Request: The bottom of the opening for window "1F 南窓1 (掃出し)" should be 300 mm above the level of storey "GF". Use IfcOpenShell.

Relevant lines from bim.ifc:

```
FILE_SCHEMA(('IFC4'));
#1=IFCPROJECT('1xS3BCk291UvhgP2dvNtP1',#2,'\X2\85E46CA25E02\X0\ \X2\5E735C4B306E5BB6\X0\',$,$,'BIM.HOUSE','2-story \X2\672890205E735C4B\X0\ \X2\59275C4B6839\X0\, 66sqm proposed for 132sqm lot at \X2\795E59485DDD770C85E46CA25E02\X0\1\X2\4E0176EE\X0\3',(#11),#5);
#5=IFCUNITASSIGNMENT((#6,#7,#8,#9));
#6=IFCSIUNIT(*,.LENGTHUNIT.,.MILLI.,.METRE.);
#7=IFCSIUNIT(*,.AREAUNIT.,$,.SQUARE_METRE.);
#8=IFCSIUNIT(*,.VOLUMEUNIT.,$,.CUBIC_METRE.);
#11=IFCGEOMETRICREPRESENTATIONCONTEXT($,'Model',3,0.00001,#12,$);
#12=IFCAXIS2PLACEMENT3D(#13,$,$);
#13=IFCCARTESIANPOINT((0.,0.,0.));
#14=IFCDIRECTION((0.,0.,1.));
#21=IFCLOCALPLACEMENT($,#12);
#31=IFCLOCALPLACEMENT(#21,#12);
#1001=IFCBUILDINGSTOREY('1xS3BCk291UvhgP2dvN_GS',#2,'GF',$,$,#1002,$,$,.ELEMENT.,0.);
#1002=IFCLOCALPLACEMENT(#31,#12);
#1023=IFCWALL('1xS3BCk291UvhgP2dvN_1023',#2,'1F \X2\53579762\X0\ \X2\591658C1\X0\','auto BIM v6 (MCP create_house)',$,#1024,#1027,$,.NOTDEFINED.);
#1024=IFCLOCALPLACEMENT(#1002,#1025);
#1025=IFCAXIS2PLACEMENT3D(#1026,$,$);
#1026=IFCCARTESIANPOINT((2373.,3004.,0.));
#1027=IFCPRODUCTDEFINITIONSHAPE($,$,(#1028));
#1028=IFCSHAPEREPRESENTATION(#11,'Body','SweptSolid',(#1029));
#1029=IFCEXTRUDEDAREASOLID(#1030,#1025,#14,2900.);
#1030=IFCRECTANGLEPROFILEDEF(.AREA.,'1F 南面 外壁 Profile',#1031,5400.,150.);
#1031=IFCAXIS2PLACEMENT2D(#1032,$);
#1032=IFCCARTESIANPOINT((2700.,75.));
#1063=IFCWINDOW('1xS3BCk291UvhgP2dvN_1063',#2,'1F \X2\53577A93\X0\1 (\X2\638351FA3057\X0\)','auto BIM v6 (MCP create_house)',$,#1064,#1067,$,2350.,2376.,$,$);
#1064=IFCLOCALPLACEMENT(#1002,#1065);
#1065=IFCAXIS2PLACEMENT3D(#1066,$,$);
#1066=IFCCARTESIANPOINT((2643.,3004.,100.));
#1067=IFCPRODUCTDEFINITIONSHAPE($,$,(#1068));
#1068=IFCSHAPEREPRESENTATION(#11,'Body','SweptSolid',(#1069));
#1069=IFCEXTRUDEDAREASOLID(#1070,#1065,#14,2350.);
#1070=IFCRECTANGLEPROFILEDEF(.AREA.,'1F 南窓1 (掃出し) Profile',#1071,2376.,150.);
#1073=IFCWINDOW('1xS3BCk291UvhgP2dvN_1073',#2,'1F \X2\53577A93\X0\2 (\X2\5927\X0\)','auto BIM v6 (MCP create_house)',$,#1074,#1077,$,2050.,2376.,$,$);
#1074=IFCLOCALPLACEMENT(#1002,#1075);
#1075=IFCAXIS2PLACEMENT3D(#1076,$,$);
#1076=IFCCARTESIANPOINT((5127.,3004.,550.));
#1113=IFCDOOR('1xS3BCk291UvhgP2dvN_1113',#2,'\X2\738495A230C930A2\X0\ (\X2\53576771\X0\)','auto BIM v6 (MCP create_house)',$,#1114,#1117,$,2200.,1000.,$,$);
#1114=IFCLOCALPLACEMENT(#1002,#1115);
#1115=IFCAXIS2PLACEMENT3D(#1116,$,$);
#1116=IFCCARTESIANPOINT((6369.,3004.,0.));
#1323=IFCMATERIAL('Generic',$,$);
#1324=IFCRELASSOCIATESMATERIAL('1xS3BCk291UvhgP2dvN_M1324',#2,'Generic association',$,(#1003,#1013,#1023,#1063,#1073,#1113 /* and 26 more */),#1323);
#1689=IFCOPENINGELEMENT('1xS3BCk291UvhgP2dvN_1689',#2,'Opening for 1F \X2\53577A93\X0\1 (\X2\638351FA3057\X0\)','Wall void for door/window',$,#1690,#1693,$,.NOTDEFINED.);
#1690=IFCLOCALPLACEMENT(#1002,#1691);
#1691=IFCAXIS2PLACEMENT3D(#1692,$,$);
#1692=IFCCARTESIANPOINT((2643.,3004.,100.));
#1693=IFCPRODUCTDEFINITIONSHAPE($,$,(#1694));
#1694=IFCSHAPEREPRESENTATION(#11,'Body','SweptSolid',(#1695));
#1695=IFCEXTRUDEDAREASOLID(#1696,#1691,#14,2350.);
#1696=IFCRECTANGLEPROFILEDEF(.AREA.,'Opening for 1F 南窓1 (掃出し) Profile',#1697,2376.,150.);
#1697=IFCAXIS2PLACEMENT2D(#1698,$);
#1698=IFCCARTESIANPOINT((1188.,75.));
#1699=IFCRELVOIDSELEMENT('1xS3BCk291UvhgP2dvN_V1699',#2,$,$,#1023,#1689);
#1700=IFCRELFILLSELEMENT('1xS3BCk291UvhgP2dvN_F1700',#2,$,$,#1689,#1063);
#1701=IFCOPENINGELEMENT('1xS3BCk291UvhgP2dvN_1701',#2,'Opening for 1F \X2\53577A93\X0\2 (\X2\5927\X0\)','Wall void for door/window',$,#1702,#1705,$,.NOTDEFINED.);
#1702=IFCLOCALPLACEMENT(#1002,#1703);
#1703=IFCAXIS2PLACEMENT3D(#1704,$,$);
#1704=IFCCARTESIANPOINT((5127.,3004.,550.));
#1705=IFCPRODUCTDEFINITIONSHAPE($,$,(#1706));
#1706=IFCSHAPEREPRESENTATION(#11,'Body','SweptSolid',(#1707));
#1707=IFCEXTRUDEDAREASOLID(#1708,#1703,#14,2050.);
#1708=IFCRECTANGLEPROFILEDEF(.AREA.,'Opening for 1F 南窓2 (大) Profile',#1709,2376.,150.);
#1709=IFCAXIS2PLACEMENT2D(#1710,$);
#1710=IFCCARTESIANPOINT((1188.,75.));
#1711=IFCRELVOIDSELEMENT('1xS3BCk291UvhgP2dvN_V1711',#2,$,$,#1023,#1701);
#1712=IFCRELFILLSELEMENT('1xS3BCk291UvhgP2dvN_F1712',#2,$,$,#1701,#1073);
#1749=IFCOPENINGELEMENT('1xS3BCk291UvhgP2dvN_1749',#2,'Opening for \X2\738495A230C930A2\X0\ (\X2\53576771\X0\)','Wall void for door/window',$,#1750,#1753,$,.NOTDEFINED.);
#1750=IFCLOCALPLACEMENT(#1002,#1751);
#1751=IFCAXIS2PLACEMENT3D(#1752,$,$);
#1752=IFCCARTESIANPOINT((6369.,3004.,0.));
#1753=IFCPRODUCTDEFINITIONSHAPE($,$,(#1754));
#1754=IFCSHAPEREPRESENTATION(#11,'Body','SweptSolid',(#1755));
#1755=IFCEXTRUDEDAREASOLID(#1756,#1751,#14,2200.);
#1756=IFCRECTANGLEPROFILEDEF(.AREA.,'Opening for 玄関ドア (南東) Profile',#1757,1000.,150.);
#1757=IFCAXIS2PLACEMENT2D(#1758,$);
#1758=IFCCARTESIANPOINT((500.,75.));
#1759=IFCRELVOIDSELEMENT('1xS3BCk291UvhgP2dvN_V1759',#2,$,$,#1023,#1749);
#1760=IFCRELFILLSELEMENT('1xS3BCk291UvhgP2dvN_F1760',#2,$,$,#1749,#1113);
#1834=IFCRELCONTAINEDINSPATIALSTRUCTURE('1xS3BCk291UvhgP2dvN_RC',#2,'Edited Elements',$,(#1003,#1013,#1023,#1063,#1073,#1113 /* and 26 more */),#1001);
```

```python
import numpy as np
import ifcopenshell
import ifcopenshell.api.geometry
import ifcopenshell.geom
import ifcopenshell.util.element
import ifcopenshell.util.placement
import ifcopenshell.util.shape
import ifcopenshell.util.unit

model = ifcopenshell.open("bim.ifc")
unit_scale = ifcopenshell.util.unit.calculate_unit_scale(model)

window = model.by_guid("1xS3BCk291UvhgP2dvN_1063")
opening = window.FillsVoids[0].RelatingOpeningElement
storey = ifcopenshell.util.element.get_container(window, ifc_class="IfcBuildingStorey")
level = ifcopenshell.util.placement.get_local_placement(storey.ObjectPlacement)[2, 3]

# The opening's origin need not be at the sill, so measure its lowest point.
shape = ifcopenshell.geom.create_shape(ifcopenshell.geom.settings(), opening)
bottom = ifcopenshell.util.shape.get_shape_bottom_elevation(shape, shape.geometry) / unit_scale
dz = level + 0.3 / unit_scale - bottom

shift = np.array([0.0, 0.0, dz])
# The window is not placed relative to its opening, so move both.
for product in (opening, window):
    matrix = ifcopenshell.util.placement.get_local_placement(product.ObjectPlacement)
    matrix[:3, 3] += shift
    ifcopenshell.api.geometry.edit_object_placement(model, product=product, matrix=matrix, is_si=False)

print(f"moved by {dz * unit_scale:+.3f} m")

model.write("bim_edited.ifc")
```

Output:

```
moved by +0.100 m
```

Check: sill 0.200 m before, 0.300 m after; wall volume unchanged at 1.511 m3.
